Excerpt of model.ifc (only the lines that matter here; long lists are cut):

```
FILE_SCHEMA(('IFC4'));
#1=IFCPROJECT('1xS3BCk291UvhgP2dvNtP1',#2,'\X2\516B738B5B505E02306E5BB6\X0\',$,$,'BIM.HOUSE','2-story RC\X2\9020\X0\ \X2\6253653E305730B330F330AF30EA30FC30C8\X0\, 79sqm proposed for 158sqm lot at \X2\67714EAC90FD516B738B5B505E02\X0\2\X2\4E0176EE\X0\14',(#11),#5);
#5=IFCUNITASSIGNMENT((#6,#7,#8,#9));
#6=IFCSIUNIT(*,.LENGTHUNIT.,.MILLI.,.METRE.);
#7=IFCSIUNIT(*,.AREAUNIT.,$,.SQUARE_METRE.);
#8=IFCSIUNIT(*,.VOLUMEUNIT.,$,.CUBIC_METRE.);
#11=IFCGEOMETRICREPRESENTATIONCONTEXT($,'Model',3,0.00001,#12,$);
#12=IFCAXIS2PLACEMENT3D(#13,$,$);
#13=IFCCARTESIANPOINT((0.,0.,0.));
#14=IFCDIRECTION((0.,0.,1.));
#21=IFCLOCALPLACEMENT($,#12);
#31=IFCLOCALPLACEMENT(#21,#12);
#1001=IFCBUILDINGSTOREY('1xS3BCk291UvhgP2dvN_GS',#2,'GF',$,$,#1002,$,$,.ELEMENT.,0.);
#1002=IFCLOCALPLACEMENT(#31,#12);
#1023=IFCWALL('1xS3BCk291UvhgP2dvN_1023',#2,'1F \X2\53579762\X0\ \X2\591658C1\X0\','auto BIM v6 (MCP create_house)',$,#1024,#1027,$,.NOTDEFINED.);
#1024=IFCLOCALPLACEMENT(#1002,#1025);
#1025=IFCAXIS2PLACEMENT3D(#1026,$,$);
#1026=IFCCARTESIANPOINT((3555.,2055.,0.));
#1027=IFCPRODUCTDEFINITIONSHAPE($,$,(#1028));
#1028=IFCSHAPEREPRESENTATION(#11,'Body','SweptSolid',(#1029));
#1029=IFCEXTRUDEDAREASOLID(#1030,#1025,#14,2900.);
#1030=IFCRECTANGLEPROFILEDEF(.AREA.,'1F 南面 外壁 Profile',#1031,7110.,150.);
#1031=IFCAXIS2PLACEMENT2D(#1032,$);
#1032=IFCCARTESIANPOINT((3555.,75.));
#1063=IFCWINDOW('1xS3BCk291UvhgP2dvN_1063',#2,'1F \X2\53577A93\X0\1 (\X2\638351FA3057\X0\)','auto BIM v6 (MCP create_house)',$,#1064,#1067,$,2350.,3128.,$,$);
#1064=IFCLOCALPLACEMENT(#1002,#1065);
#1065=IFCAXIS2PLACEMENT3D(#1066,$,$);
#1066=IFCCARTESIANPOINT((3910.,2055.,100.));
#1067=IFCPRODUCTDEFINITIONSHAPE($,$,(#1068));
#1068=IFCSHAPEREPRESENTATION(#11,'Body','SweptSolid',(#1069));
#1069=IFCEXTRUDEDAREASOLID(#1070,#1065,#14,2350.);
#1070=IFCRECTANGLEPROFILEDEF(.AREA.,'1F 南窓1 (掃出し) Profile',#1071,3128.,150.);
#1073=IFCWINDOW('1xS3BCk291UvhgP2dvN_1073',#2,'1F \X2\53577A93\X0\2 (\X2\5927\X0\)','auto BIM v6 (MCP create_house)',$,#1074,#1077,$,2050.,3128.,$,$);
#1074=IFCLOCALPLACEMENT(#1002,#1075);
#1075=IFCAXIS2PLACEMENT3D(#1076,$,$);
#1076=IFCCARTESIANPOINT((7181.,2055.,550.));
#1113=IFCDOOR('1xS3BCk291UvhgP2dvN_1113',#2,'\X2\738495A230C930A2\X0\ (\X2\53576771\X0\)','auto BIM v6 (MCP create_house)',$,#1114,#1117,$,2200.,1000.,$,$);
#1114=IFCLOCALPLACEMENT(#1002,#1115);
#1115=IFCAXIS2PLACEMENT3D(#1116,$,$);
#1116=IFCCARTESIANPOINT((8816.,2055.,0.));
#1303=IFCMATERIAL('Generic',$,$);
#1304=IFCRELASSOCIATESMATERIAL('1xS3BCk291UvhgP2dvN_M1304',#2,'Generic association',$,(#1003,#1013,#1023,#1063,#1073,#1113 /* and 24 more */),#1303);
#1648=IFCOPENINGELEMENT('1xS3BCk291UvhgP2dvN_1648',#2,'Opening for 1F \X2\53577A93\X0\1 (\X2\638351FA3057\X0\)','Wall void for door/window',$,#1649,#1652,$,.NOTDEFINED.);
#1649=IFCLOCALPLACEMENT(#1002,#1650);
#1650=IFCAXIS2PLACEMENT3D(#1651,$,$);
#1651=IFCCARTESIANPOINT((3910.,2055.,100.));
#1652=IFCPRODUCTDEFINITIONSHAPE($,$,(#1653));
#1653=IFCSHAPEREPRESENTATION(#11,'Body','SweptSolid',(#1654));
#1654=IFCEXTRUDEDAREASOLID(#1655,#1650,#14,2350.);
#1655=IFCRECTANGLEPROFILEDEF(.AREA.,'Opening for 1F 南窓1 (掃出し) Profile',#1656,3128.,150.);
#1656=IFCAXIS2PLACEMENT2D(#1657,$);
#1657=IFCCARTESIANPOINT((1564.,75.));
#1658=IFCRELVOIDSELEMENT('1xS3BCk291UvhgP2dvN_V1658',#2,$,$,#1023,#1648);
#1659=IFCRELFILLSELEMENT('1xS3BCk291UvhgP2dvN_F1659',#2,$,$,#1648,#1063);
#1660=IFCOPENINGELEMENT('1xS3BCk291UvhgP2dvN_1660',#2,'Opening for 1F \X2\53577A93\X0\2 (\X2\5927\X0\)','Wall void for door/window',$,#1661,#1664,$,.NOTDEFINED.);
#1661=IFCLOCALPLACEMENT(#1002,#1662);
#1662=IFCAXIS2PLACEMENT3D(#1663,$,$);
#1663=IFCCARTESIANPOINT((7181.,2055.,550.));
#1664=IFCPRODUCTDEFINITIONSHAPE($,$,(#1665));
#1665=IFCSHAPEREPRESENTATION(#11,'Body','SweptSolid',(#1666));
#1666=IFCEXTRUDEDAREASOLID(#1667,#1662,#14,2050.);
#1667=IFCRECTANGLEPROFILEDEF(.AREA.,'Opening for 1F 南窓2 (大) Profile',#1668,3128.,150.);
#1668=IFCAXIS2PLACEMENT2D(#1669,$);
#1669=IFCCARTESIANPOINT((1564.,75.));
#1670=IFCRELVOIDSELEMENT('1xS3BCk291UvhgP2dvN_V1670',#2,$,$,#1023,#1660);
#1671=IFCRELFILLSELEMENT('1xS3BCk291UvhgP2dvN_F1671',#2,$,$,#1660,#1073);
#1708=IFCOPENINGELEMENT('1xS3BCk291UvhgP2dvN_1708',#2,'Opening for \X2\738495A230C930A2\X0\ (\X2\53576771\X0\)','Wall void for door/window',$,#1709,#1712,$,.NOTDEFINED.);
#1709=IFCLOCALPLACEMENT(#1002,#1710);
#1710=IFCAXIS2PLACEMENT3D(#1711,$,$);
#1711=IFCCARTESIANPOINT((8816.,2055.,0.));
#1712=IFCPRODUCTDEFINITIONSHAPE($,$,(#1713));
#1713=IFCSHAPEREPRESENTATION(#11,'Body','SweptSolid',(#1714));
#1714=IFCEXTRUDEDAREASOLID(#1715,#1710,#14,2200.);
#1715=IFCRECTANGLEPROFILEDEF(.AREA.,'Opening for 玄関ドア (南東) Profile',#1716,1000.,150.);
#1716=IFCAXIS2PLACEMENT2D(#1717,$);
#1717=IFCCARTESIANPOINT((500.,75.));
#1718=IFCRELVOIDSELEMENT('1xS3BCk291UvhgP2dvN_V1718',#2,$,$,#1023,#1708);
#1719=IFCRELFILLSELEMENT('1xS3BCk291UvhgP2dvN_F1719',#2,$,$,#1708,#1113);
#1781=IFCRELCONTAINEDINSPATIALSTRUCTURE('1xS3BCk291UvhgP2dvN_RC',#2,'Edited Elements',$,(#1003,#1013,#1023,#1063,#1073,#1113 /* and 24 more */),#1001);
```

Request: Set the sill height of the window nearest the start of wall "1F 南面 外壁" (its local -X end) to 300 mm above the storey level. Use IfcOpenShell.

```python
import numpy as np
import ifcopenshell
import ifcopenshell.api.geometry
import ifcopenshell.geom
import ifcopenshell.util.element
import ifcopenshell.util.placement
import ifcopenshell.util.shape
import ifcopenshell.util.unit

model = ifcopenshell.open("model.ifc")
unit_scale = ifcopenshell.util.unit.calculate_unit_scale(model)

window = model.by_guid("1xS3BCk291UvhgP2dvN_1063")
opening = window.FillsVoids[0].RelatingOpeningElement
storey = ifcopenshell.util.element.get_container(window, ifc_class="IfcBuildingStorey")
level = ifcopenshell.util.placement.get_local_placement(storey.ObjectPlacement)[2, 3]

# The opening's origin need not be at the sill, so measure its lowest point.
shape = ifcopenshell.geom.create_shape(ifcopenshell.geom.settings(), opening)
bottom = ifcopenshell.util.shape.get_shape_bottom_elevation(shape, shape.geometry) / unit_scale
dz = level + 0.3 / unit_scale - bottom

shift = np.array([0.0, 0.0, dz])
# The window is not placed relative to its opening, so move both.
for product in (opening, window):
    matrix = ifcopenshell.util.placement.get_local_placement(product.ObjectPlacement)
    matrix[:3, 3] += shift
    ifcopenshell.api.geometry.edit_object_placement(model, product=product, matrix=matrix, is_si=False)

print(f"moved by {dz * unit_scale:+.3f} m")

model.write("model_v2.ifc")
```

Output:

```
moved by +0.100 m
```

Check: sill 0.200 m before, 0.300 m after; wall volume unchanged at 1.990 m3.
